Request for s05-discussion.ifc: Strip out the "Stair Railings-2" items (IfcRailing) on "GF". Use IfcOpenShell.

First a look at what the model holds.

```python
import ifcopenshell
import ifcopenshell.util.element

model = ifcopenshell.open("s05-discussion.ifc")
print(model.schema)
storey = next(s for s in model.by_type("IfcBuildingStorey") if s.Name == "GF")
railings = [e for e in ifcopenshell.util.element.get_decomposition(storey) if e.is_a("IfcRailing")]
seen = {}
for e in railings:
    element_type = ifcopenshell.util.element.get_type(e)
    name = element_type.Name if element_type not in (None, e) else None
    seen[name] = seen.get(name, 0) + 1
for name, count in sorted(seen.items(), key=str):
    print(count, "x", name)
```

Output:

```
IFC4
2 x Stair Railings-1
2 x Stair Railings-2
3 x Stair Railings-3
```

```python
import ifcopenshell
import ifcopenshell.api.root
import ifcopenshell.util.element

model = ifcopenshell.open("s05-discussion.ifc")

storey = next(s for s in model.by_type("IfcBuildingStorey") if s.Name == "GF")
railings = [e for e in ifcopenshell.util.element.get_decomposition(storey) if e.is_a("IfcRailing")]
targets = [e for e in railings if (t := ifcopenshell.util.element.get_type(e)) not in (None, e) and t.Name == "Stair Railings-2"]

for e in targets:
    ifcopenshell.api.root.remove_product(model, product=e)
print(len(targets), "removed")

model.write("s05-discussion_edited.ifc")
```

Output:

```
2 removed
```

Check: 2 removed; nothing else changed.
